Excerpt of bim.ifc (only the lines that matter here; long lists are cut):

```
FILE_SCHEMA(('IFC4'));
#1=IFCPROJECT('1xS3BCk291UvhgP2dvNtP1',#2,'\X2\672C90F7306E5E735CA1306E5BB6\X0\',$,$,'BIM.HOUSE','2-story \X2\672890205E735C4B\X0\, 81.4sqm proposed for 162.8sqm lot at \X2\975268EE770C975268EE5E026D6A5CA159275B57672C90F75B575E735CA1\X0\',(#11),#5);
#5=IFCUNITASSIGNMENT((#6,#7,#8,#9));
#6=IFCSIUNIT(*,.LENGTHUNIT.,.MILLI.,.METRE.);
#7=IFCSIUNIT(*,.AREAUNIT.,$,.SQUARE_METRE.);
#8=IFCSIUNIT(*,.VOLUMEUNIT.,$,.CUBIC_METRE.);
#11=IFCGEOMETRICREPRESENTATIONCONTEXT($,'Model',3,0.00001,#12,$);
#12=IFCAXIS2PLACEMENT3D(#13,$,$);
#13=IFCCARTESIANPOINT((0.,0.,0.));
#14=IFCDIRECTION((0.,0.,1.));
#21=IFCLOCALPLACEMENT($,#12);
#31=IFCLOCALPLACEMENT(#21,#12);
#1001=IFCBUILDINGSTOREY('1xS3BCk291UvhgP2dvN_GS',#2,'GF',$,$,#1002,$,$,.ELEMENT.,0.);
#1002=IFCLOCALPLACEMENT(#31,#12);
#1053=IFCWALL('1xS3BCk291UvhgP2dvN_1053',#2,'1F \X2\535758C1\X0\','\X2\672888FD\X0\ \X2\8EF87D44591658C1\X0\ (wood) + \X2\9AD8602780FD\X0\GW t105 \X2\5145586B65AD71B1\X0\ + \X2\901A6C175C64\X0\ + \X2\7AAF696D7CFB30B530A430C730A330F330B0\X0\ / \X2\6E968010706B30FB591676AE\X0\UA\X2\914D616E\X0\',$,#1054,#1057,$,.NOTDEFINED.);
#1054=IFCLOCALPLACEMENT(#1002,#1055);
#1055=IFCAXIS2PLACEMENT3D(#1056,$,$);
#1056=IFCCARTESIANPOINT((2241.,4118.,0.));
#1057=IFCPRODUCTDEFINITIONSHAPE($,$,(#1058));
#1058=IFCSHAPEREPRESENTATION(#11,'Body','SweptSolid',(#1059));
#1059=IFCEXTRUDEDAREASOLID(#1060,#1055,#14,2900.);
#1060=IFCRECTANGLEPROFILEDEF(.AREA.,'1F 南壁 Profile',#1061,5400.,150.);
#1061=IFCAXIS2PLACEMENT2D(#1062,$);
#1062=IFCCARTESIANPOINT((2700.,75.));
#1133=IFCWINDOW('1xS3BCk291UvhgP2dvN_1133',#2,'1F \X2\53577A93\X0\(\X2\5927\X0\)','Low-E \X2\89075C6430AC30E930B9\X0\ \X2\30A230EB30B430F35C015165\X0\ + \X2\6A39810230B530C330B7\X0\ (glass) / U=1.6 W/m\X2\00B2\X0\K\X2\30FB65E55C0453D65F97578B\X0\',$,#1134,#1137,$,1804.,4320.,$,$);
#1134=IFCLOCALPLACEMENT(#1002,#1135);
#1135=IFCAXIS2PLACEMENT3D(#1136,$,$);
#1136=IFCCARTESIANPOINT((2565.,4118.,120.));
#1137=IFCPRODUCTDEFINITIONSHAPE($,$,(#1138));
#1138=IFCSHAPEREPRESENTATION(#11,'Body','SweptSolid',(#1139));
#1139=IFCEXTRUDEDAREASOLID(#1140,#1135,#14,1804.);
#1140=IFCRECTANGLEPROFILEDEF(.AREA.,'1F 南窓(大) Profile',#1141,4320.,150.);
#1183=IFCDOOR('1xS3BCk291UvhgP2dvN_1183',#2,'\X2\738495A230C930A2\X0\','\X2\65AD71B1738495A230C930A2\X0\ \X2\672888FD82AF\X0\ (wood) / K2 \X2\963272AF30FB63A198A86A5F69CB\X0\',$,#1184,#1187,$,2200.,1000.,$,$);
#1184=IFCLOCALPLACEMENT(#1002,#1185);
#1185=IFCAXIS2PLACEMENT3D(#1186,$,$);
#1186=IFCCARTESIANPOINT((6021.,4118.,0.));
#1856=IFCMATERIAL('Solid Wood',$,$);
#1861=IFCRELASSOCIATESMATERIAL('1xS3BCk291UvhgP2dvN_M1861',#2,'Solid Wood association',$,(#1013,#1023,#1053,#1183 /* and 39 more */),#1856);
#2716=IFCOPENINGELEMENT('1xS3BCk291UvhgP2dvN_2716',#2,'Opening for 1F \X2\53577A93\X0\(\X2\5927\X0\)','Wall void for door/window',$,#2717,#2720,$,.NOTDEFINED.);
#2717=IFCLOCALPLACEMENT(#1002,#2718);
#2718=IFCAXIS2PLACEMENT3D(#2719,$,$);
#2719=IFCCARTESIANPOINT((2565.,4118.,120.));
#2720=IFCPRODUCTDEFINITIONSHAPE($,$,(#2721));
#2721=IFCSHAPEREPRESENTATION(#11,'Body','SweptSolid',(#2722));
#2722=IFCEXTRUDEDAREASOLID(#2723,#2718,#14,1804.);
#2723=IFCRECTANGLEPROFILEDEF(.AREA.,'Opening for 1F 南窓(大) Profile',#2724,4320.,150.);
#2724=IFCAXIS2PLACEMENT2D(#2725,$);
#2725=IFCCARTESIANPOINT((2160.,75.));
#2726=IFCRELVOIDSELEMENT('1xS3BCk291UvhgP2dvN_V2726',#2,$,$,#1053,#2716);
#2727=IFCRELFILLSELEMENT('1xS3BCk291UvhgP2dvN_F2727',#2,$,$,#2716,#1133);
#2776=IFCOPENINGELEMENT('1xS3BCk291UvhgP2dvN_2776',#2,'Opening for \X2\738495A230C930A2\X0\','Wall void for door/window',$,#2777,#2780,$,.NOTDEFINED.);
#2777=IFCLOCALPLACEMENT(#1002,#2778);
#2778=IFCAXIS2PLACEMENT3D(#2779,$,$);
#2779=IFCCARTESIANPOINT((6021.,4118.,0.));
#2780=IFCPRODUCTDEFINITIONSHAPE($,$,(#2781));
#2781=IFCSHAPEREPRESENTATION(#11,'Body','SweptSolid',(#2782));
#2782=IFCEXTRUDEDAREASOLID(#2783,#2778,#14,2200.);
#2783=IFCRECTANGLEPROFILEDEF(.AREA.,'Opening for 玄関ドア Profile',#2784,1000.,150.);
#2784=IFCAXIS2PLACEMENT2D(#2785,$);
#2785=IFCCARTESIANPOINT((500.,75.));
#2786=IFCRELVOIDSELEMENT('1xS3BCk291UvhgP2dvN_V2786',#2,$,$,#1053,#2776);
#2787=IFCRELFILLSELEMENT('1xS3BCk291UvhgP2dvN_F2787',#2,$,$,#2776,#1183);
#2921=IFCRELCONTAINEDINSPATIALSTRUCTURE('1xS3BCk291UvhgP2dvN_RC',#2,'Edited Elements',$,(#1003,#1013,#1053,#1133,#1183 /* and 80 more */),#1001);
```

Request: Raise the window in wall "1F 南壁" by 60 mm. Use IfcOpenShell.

```python
import numpy as np
import ifcopenshell
import ifcopenshell.api.geometry
import ifcopenshell.util.placement
import ifcopenshell.util.unit

model = ifcopenshell.open("bim.ifc")
unit_scale = ifcopenshell.util.unit.calculate_unit_scale(model)

window = model.by_id(1133)
opening = window.FillsVoids[0].RelatingOpeningElement
dz = 0.06 / unit_scale

shift = np.array([0.0, 0.0, dz])
# The window is not placed relative to its opening, so move both.
for product in (opening, window):
    matrix = ifcopenshell.util.placement.get_local_placement(product.ObjectPlacement)
    matrix[:3, 3] += shift
    ifcopenshell.api.geometry.edit_object_placement(model, product=product, matrix=matrix, is_si=False)

print(f"moved by {dz * unit_scale:+.3f} m")

model.write("bim-out.ifc")
```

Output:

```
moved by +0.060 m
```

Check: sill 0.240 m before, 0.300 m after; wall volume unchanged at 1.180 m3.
